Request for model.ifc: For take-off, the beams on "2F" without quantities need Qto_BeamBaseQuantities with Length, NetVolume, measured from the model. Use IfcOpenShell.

First a look at what the model holds.

```python
import ifcopenshell
import ifcopenshell.util.element
import ifcopenshell.util.unit

model = ifcopenshell.open("model.ifc")
print(model.schema)
for unit_type in ("LENGTHUNIT", "AREAUNIT", "VOLUMEUNIT"):
    print(unit_type, ifcopenshell.util.unit.calculate_unit_scale(model, unit_type))
storey = next(s for s in model.by_type("IfcBuildingStorey") if s.Name == "2F")
beams = [e for e in ifcopenshell.util.element.get_decomposition(storey) if e.is_a("IfcBeam")]
for e in sorted(beams, key=lambda e: e.id()):
    print(e.id(), e.is_a(), e.Name, list(ifcopenshell.util.element.get_psets(e, qtos_only=True)), sep=" | ")
```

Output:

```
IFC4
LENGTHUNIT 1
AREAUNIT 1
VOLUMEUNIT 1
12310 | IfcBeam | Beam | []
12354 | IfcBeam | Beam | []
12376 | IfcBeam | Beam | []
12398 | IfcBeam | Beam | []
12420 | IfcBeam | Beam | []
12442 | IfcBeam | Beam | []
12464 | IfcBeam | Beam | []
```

```python
import ifcopenshell
import ifcopenshell.api.pset
import ifcopenshell.geom
import ifcopenshell.util.element
import ifcopenshell.util.shape
import ifcopenshell.util.unit

model = ifcopenshell.open("model.ifc")
unit_scale = ifcopenshell.util.unit.calculate_unit_scale(model)
volume_scale = ifcopenshell.util.unit.calculate_unit_scale(model, "VOLUMEUNIT")
settings = ifcopenshell.geom.settings()

storey = next(s for s in model.by_type("IfcBuildingStorey") if s.Name == "2F")
beams = [e for e in ifcopenshell.util.element.get_decomposition(storey) if e.is_a("IfcBeam")]

for e in sorted(beams, key=lambda e: e.id()):
    if ifcopenshell.util.element.get_psets(e, qtos_only=True, should_inherit=False):
        continue
    # Geometry comes back in metres, in the element's own axes.
    shape = ifcopenshell.geom.create_shape(settings, e)
    values = {
        "Length": ifcopenshell.util.shape.get_max_xyz(shape.geometry) / unit_scale,
        "NetVolume": ifcopenshell.util.shape.get_volume(shape.geometry) / volume_scale,
    }
    qto = ifcopenshell.api.pset.add_qto(model, product=e, name="Qto_BeamBaseQuantities")
    ifcopenshell.api.pset.edit_qto(model, qto=qto, properties=values)
    print(e.id(), {k: round(v, 3) for k, v in values.items()})

model.write("model_edited.ifc")
```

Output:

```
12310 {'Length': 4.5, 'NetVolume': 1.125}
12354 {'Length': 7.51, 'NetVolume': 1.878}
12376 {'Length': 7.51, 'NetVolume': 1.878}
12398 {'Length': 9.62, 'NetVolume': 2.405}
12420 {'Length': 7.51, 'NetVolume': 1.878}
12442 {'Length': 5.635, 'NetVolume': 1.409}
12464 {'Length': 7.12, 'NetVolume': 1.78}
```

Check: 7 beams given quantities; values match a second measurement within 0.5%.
